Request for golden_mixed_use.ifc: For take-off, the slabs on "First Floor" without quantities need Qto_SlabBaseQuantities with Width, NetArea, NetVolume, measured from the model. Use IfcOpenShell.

First a look at what the model holds.

```python
import ifcopenshell
import ifcopenshell.util.element
import ifcopenshell.util.unit

model = ifcopenshell.open("golden_mixed_use.ifc")
print(model.schema)
for unit_type in ("LENGTHUNIT", "AREAUNIT", "VOLUMEUNIT"):
    print(unit_type, ifcopenshell.util.unit.calculate_unit_scale(model, unit_type))
storey = next(s for s in model.by_type("IfcBuildingStorey") if s.Name == "First Floor")
slabs = [e for e in ifcopenshell.util.element.get_decomposition(storey) if e.is_a("IfcSlab")]
for e in sorted(slabs, key=lambda e: e.id()):
    print(e.id(), e.is_a(), e.Name, list(ifcopenshell.util.element.get_psets(e, qtos_only=True)), sep=" | ")
```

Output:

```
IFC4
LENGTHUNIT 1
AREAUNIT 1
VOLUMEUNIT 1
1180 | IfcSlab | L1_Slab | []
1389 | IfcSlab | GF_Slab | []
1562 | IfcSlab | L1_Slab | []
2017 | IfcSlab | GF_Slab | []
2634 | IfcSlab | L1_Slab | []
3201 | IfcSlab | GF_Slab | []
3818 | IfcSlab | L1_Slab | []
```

```python
import ifcopenshell
import ifcopenshell.api.pset
import ifcopenshell.geom
import ifcopenshell.util.element
import ifcopenshell.util.shape
import ifcopenshell.util.unit

model = ifcopenshell.open("golden_mixed_use.ifc")
unit_scale = ifcopenshell.util.unit.calculate_unit_scale(model)
area_scale = ifcopenshell.util.unit.calculate_unit_scale(model, "AREAUNIT")
volume_scale = ifcopenshell.util.unit.calculate_unit_scale(model, "VOLUMEUNIT")
settings = ifcopenshell.geom.settings()

storey = next(s for s in model.by_type("IfcBuildingStorey") if s.Name == "First Floor")
slabs = [e for e in ifcopenshell.util.element.get_decomposition(storey) if e.is_a("IfcSlab")]

for e in sorted(slabs, key=lambda e: e.id()):
    if ifcopenshell.util.element.get_psets(e, qtos_only=True, should_inherit=False):
        continue
    # Geometry comes back in metres, in the element's own axes.
    shape = ifcopenshell.geom.create_shape(settings, e)
    values = {
        "Width": ifcopenshell.util.shape.get_z(shape.geometry) / unit_scale,
        "NetArea": ifcopenshell.util.shape.get_footprint_area(shape.geometry) / area_scale,
        "NetVolume": ifcopenshell.util.shape.get_volume(shape.geometry) / volume_scale,
    }
    qto = ifcopenshell.api.pset.add_qto(model, product=e, name="Qto_SlabBaseQuantities")
    ifcopenshell.api.pset.edit_qto(model, qto=qto, properties=values)
    print(e.id(), {k: round(v, 3) for k, v in values.items()})

model.write("golden_mixed_use_edited.ifc")
```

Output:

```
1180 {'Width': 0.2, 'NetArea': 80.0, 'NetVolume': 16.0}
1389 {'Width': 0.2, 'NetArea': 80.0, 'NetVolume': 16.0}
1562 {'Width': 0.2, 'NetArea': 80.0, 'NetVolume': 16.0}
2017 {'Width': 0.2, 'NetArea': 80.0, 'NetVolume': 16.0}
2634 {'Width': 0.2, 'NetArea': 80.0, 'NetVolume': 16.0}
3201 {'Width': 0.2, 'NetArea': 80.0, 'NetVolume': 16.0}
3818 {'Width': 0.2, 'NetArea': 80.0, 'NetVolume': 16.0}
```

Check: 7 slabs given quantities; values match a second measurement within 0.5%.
